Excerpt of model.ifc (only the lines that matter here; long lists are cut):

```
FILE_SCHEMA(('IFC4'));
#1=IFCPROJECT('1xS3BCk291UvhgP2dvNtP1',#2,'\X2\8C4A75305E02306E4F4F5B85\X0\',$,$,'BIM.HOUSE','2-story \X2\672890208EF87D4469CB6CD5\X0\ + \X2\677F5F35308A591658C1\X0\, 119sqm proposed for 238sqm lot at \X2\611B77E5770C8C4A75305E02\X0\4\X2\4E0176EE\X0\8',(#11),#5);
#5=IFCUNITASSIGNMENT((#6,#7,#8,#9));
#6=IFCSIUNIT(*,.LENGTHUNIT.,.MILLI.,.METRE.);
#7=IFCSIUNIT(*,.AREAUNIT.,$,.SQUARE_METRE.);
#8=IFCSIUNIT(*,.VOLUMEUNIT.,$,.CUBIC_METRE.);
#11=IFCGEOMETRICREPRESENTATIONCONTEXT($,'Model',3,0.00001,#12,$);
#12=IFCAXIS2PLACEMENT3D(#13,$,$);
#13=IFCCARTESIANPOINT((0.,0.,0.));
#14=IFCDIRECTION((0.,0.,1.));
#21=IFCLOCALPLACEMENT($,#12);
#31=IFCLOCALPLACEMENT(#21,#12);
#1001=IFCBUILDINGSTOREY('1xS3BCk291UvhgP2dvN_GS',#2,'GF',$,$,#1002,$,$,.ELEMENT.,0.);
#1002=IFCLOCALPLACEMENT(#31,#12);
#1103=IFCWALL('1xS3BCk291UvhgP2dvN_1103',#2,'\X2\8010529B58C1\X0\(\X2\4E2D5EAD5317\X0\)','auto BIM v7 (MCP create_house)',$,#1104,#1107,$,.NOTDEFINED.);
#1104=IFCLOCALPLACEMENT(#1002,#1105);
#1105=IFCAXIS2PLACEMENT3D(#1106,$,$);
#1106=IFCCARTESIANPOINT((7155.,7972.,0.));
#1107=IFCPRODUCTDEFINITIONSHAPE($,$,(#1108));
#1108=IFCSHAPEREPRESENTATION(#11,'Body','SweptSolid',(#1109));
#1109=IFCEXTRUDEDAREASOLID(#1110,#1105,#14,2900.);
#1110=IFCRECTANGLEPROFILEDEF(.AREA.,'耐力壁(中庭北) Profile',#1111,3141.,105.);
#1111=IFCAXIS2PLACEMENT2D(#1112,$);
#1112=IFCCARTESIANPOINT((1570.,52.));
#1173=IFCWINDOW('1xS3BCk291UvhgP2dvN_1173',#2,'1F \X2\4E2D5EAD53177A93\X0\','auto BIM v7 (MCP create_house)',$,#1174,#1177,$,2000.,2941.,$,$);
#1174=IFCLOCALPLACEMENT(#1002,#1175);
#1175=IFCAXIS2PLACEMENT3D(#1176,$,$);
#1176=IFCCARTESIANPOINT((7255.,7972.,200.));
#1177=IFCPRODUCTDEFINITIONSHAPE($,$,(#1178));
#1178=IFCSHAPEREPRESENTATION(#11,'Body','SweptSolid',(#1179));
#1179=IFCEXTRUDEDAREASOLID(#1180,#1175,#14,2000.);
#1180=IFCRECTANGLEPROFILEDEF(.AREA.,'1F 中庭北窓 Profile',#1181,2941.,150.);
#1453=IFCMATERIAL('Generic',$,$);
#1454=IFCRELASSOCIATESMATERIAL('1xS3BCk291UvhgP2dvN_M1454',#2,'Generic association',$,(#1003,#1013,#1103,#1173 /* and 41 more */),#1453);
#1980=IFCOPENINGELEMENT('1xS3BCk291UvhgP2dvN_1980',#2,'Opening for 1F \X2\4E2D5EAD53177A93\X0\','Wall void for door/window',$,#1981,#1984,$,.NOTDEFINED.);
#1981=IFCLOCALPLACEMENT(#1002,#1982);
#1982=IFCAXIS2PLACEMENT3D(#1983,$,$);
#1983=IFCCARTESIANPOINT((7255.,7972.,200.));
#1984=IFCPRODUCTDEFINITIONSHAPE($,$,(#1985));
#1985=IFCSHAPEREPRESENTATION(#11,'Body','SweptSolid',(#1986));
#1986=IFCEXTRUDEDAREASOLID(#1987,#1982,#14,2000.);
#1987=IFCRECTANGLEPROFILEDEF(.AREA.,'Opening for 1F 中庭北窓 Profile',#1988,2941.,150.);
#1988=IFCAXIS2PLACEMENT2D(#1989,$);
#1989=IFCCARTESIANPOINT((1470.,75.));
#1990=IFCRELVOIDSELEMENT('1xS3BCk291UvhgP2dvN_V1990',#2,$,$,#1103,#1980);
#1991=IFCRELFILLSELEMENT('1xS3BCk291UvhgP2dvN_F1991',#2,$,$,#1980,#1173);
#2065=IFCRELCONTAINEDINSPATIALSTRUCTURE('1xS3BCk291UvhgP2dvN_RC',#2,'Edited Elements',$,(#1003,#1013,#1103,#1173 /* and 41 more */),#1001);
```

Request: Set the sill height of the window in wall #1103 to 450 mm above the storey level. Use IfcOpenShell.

```python
import numpy as np
import ifcopenshell
import ifcopenshell.api.geometry
import ifcopenshell.geom
import ifcopenshell.util.element
import ifcopenshell.util.placement
import ifcopenshell.util.shape
import ifcopenshell.util.unit

model = ifcopenshell.open("model.ifc")
unit_scale = ifcopenshell.util.unit.calculate_unit_scale(model)

window = model.by_guid("1xS3BCk291UvhgP2dvN_1173")
opening = window.FillsVoids[0].RelatingOpeningElement
storey = ifcopenshell.util.element.get_container(window, ifc_class="IfcBuildingStorey")
level = ifcopenshell.util.placement.get_local_placement(storey.ObjectPlacement)[2, 3]

# The opening's origin need not be at the sill, so measure its lowest point.
shape = ifcopenshell.geom.create_shape(ifcopenshell.geom.settings(), opening)
bottom = ifcopenshell.util.shape.get_shape_bottom_elevation(shape, shape.geometry) / unit_scale
dz = level + 0.45 / unit_scale - bottom

shift = np.array([0.0, 0.0, dz])
# The window is not placed relative to its opening, so move both.
for product in (opening, window):
    matrix = ifcopenshell.util.placement.get_local_placement(product.ObjectPlacement)
    matrix[:3, 3] += shift
    ifcopenshell.api.geometry.edit_object_placement(model, product=product, matrix=matrix, is_si=False)

print(f"moved by {dz * unit_scale:+.3f} m")

model.write("model-out.ifc")
```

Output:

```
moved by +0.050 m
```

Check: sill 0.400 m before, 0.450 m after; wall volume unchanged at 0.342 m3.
